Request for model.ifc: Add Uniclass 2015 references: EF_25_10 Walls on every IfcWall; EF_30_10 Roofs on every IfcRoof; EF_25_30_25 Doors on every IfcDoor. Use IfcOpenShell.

First a look at what the model holds.

```python
import ifcopenshell

model = ifcopenshell.open("model.ifc")
print(model.schema)
print("classifications:", [c.Name for c in model.by_type("IfcClassification")])
for ifc_class in ("IfcDoor", "IfcRoof", "IfcStair", "IfcWall", "IfcWindow"):
    print(ifc_class, len(model.by_type(ifc_class)))
```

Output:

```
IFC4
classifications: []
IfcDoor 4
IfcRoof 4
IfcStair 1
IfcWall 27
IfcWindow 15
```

```python
import ifcopenshell
import ifcopenshell.api.classification

model = ifcopenshell.open("model.ifc")

system = ifcopenshell.api.classification.add_classification(model, classification="Uniclass 2015")

codes = {
    "IfcWall": ("EF_25_10", "Walls"),
    "IfcRoof": ("EF_30_10", "Roofs"),
    "IfcDoor": ("EF_25_30_25", "Doors"),
}
for ifc_class, (code, name) in codes.items():
    products = model.by_type(ifc_class)
    ifcopenshell.api.classification.add_reference(
        model, products=products, classification=system, identification=code, name=name
    )
    print(code, len(products))

model.write("model_updated.ifc")
```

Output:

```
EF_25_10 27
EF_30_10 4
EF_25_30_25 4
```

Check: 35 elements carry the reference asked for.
